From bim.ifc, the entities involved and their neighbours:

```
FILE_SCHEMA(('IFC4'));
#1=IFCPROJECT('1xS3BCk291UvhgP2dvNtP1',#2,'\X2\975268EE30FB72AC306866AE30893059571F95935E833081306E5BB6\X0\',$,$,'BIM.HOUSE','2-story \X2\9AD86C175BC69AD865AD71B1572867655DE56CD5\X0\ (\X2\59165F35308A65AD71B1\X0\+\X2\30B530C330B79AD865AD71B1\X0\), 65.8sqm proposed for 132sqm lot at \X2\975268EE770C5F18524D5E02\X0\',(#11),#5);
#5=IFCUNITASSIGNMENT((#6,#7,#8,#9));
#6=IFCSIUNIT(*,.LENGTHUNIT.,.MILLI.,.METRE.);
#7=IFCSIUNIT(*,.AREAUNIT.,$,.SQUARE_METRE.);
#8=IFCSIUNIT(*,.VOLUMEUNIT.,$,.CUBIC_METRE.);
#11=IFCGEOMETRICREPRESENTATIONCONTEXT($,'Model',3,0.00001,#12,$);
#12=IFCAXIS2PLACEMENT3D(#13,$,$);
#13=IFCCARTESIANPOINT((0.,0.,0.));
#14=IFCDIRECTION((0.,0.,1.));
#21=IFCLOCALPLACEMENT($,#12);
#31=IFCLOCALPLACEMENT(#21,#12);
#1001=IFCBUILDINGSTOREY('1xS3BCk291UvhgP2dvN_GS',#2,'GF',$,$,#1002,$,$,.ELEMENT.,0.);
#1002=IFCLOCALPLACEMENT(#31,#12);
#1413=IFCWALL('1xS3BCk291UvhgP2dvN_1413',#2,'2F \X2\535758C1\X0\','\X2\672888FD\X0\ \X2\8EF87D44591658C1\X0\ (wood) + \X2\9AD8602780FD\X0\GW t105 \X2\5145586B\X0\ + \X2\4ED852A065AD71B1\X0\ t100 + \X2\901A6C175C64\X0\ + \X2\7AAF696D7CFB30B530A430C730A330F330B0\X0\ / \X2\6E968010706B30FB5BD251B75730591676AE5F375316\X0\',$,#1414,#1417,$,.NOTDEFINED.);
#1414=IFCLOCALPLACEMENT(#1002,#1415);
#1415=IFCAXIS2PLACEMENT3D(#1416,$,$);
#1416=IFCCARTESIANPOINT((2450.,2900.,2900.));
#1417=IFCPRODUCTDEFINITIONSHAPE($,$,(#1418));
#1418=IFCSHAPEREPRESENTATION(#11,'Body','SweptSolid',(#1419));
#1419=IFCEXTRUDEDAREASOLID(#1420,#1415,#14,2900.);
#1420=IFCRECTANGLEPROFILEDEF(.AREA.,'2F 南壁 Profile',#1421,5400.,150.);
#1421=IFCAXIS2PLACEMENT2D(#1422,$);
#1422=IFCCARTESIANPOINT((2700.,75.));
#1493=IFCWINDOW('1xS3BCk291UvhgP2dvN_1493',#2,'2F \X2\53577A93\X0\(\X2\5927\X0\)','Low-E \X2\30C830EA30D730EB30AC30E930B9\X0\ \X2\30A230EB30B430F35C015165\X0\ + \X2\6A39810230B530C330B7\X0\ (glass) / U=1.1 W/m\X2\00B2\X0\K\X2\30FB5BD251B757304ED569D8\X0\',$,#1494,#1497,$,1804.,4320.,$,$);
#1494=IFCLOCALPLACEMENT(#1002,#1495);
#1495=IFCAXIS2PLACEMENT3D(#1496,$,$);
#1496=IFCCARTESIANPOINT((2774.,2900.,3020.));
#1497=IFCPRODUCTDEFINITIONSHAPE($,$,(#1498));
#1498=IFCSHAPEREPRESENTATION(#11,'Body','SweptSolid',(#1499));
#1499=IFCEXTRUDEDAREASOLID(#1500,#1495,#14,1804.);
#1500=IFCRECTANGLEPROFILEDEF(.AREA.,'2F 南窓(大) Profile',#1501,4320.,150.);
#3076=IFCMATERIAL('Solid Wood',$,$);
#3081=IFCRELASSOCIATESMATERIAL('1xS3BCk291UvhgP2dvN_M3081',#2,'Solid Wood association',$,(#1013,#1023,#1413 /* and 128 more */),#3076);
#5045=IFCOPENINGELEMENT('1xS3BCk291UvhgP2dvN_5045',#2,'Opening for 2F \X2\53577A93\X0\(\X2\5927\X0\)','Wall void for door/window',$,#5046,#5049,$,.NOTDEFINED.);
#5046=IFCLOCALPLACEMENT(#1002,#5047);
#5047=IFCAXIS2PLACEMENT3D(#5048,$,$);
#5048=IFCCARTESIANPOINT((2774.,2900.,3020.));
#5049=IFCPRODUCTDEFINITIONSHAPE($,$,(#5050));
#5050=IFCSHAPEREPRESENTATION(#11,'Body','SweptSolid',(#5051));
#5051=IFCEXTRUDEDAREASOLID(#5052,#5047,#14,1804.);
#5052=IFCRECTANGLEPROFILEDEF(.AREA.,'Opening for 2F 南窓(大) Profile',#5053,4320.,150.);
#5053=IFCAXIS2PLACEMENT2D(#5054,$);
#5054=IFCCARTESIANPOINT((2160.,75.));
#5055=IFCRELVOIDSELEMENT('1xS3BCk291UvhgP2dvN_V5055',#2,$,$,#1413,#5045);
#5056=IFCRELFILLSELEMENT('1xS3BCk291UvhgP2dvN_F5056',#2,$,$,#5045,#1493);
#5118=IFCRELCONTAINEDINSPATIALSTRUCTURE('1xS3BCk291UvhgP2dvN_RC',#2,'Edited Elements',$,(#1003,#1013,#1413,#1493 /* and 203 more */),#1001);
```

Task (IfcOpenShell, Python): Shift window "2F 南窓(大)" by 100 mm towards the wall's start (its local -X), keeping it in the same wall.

```python
import ifcopenshell
import ifcopenshell.api.geometry
import ifcopenshell.util.placement

model = ifcopenshell.open("bim.ifc")

window = model.by_guid("1xS3BCk291UvhgP2dvN_1493")
opening = window.FillsVoids[0].RelatingOpeningElement
wall = opening.VoidsElements[0].RelatingBuildingElement

wall_matrix = ifcopenshell.util.placement.get_local_placement(wall.ObjectPlacement)
shift = wall_matrix[:3, 0] * -100.0
before = ifcopenshell.util.placement.get_local_placement(window.ObjectPlacement)[:3, 3].copy()

# The window is not placed relative to its opening, so move both.
for product in (opening, window):
    matrix = ifcopenshell.util.placement.get_local_placement(product.ObjectPlacement)
    matrix[:3, 3] += shift
    ifcopenshell.api.geometry.edit_object_placement(model, product=product, matrix=matrix, is_si=False)

after = ifcopenshell.util.placement.get_local_placement(window.ObjectPlacement)[:3, 3]
print("window moved by", (after - before).round(3) + 0.0)

model.write("bim_v2.ifc")
```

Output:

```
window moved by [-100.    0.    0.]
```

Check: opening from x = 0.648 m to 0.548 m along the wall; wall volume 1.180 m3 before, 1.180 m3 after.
